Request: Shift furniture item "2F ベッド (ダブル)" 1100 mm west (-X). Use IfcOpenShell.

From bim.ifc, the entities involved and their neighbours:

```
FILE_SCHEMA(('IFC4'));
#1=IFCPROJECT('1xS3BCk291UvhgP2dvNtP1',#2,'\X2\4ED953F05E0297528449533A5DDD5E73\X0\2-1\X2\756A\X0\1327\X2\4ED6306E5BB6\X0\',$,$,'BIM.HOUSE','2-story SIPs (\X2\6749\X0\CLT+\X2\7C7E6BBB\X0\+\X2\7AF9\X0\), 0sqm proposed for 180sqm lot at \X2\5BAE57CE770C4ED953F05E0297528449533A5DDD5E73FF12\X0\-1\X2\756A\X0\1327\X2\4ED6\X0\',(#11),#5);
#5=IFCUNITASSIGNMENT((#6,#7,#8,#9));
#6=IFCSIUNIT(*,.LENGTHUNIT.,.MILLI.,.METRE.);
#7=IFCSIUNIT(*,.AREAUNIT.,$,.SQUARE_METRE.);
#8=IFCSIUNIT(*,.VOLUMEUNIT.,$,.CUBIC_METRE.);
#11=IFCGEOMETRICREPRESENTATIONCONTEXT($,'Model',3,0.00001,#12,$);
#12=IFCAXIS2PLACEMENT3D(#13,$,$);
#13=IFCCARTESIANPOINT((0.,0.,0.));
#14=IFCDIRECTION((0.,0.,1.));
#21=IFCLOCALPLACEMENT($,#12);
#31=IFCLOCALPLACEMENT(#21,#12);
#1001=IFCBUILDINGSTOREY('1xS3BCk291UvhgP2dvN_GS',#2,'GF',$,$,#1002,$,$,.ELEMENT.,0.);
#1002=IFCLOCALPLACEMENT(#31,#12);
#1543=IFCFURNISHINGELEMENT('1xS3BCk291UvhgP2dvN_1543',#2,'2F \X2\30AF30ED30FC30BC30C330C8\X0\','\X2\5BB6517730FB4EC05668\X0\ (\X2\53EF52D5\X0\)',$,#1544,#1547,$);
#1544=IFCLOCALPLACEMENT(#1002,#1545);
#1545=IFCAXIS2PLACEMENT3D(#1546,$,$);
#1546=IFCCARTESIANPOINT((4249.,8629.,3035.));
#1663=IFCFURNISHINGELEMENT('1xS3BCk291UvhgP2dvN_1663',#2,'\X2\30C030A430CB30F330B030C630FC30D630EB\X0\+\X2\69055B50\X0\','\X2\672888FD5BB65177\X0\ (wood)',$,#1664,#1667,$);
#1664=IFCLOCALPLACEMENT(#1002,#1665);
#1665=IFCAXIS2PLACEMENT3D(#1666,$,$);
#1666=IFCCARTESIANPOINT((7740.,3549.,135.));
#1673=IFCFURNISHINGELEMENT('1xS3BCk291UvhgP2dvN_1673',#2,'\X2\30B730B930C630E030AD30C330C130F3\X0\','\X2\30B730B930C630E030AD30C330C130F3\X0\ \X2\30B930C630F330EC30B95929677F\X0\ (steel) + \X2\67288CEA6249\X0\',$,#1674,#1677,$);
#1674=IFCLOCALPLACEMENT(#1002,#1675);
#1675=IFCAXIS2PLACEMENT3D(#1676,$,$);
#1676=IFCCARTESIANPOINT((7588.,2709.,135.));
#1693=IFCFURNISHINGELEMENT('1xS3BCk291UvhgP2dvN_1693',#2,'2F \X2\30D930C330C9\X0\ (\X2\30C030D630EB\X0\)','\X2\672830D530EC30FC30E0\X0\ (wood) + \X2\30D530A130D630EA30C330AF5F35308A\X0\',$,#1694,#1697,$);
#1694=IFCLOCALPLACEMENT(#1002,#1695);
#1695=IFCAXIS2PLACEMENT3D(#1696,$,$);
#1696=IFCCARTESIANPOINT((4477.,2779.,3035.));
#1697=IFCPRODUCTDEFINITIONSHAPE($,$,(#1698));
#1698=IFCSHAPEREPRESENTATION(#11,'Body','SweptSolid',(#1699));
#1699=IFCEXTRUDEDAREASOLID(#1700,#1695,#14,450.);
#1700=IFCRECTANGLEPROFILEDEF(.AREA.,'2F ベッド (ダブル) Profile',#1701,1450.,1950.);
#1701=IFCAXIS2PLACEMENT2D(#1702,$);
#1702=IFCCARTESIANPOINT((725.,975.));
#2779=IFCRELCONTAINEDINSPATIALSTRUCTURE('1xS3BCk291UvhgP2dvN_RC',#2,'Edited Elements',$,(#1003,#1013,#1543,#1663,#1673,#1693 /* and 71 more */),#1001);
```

```python
import ifcopenshell
import ifcopenshell.api.geometry
import ifcopenshell.util.placement
import ifcopenshell.util.unit

model = ifcopenshell.open("bim.ifc")
unit_scale = ifcopenshell.util.unit.calculate_unit_scale(model)

item = model.by_guid("1xS3BCk291UvhgP2dvN_1693")
matrix = ifcopenshell.util.placement.get_local_placement(item.ObjectPlacement)
matrix[0, 3] -= 1.1 / unit_scale
ifcopenshell.api.geometry.edit_object_placement(model, product=item, matrix=matrix, is_si=False)

print(ifcopenshell.util.placement.get_local_placement(item.ObjectPlacement).round(3) + 0.0)

model.write("bim_v2.ifc")
```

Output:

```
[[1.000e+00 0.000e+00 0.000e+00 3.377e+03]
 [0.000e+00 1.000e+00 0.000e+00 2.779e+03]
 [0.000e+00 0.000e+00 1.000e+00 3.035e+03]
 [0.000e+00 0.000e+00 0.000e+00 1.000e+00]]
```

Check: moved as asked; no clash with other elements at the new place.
